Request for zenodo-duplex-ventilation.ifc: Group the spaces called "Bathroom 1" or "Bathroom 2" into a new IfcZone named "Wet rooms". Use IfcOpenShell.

First a look at what the model holds.

```python
import ifcopenshell

model = ifcopenshell.open("zenodo-duplex-ventilation.ifc")
print(model.schema)
seen = {}
for space in model.by_type("IfcSpace"):
    seen[space.LongName] = seen.get(space.LongName, 0) + 1
for name, count in sorted(seen.items(), key=str):
    print(count, "x", name)
print("zones:", [z.Name for z in model.by_type("IfcZone")][:20])
```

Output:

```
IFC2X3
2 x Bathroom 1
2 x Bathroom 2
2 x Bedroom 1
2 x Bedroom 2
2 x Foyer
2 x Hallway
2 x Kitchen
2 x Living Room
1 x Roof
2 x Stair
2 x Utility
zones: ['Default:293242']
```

```python
import ifcopenshell
import ifcopenshell.api.group
import ifcopenshell.api.root

model = ifcopenshell.open("zenodo-duplex-ventilation.ifc")

names = {"Bathroom 1", "Bathroom 2"}
spaces = [s for s in model.by_type("IfcSpace") if s.LongName in names]

zone = ifcopenshell.api.root.create_entity(model, ifc_class="IfcZone", name="Wet rooms")
ifcopenshell.api.group.assign_group(model, products=spaces, group=zone)
print(len(spaces), "spaces in", zone.Name)

model.write("zenodo-duplex-ventilation-out.ifc")
```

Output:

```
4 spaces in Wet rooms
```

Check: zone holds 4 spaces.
